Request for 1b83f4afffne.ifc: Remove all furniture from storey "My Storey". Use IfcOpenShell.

First a look at what the model holds.

```python
import ifcopenshell
import ifcopenshell.util.element

model = ifcopenshell.open("1b83f4afffne.ifc")
print(model.schema)
storey = next(s for s in model.by_type("IfcBuildingStorey") if s.Name == "My Storey")
furniture = [e for e in ifcopenshell.util.element.get_decomposition(storey) if e.is_a("IfcFurnishingElement")]
seen = {}
for e in furniture:
    element_type = ifcopenshell.util.element.get_type(e)
    name = element_type.Name if element_type not in (None, e) else None
    seen[name] = seen.get(name, 0) + 1
for name, count in sorted(seen.items(), key=str):
    print(count, "x", name)
```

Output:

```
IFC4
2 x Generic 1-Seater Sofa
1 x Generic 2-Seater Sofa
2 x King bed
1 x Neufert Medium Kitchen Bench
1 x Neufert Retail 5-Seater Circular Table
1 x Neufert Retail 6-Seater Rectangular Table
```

```python
import ifcopenshell
import ifcopenshell.api.root
import ifcopenshell.util.element

model = ifcopenshell.open("1b83f4afffne.ifc")

storey = next(s for s in model.by_type("IfcBuildingStorey") if s.Name == "My Storey")
furniture = [e for e in ifcopenshell.util.element.get_decomposition(storey) if e.is_a("IfcFurnishingElement")]

for e in furniture:
    ifcopenshell.api.root.remove_product(model, product=e)
print(len(furniture), "removed")

model.write("1b83f4afffne_v2.ifc")
```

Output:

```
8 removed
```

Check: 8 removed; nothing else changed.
